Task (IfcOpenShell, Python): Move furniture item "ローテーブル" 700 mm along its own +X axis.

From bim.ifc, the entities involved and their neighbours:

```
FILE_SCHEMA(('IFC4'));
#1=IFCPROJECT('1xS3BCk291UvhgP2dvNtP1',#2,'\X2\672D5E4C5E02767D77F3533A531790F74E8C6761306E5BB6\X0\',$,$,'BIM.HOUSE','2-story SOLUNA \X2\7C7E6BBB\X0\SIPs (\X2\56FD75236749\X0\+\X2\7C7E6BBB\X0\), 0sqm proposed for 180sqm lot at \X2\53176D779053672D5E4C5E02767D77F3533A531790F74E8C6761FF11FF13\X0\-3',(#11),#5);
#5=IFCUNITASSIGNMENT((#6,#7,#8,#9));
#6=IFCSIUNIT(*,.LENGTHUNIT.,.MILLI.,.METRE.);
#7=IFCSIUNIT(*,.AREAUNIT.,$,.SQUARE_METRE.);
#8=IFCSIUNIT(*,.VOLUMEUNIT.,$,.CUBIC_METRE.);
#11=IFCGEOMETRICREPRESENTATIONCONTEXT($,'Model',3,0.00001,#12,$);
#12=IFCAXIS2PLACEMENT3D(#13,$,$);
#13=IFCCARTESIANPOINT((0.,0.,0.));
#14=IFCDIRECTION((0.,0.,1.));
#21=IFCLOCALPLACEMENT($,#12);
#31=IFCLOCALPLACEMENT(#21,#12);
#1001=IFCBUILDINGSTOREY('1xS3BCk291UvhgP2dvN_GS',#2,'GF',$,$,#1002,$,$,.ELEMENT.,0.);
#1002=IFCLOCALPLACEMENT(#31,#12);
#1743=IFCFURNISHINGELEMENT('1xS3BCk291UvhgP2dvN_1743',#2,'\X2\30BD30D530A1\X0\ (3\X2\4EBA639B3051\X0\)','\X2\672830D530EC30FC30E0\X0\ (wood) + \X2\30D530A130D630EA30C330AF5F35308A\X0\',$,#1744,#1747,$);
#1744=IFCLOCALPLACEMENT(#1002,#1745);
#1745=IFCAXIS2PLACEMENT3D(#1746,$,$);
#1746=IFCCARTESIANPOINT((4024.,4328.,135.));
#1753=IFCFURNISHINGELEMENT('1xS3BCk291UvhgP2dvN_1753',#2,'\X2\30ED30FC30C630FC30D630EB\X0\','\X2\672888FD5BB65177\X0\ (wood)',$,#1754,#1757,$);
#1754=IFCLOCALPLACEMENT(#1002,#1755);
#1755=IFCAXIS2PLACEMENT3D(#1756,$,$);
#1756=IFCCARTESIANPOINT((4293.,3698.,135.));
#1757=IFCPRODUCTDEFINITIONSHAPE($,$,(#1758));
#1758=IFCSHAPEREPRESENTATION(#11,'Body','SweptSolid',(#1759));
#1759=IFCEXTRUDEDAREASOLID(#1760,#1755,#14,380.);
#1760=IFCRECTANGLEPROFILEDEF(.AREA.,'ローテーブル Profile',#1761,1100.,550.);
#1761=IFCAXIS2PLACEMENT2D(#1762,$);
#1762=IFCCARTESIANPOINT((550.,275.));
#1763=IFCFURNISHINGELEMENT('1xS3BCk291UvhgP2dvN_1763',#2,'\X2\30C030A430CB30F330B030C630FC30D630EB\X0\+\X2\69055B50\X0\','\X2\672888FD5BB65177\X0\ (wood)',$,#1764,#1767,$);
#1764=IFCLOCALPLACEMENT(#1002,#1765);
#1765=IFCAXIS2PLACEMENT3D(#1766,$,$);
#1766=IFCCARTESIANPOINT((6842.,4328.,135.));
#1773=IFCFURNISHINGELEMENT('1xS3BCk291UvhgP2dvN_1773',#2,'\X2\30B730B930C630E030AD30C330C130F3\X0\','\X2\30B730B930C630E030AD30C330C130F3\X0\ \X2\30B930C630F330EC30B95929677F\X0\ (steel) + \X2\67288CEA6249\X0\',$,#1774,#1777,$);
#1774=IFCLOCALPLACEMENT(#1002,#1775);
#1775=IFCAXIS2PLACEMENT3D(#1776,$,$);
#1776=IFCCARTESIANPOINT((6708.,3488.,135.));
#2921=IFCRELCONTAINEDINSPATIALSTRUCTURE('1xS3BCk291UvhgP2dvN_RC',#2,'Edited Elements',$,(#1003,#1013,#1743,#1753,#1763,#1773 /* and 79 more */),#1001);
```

```python
import ifcopenshell
import ifcopenshell.api.geometry
import ifcopenshell.util.placement
import ifcopenshell.util.unit

model = ifcopenshell.open("bim.ifc")
unit_scale = ifcopenshell.util.unit.calculate_unit_scale(model)

item = model.by_guid("1xS3BCk291UvhgP2dvN_1753")
matrix = ifcopenshell.util.placement.get_local_placement(item.ObjectPlacement)
matrix[:3, 3] += matrix[:3, 0] * 0.7 / unit_scale
ifcopenshell.api.geometry.edit_object_placement(model, product=item, matrix=matrix, is_si=False)

print(ifcopenshell.util.placement.get_local_placement(item.ObjectPlacement).round(3) + 0.0)

model.write("bim_edited.ifc")
```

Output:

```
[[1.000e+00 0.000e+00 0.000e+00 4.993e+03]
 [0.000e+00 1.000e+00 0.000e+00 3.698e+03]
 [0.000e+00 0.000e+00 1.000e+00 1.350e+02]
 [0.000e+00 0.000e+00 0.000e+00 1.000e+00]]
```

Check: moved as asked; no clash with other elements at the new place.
